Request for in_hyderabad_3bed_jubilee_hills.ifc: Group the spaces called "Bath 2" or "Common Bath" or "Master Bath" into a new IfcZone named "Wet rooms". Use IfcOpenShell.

First a look at what the model holds.

```python
import ifcopenshell

model = ifcopenshell.open("in_hyderabad_3bed_jubilee_hills.ifc")
print(model.schema)
seen = {}
for space in model.by_type("IfcSpace"):
    seen[space.LongName] = seen.get(space.LongName, 0) + 1
for name, count in sorted(seen.items(), key=str):
    print(count, "x", name)
print("zones:", [z.Name for z in model.by_type("IfcZone")][:20])
```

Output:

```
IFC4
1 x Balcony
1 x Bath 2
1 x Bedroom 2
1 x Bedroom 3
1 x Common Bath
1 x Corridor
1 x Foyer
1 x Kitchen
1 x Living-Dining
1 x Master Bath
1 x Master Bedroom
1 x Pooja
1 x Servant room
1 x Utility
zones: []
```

```python
import ifcopenshell
import ifcopenshell.api.group
import ifcopenshell.api.root

model = ifcopenshell.open("in_hyderabad_3bed_jubilee_hills.ifc")

names = {"Bath 2", "Common Bath", "Master Bath"}
spaces = [s for s in model.by_type("IfcSpace") if s.LongName in names]

zone = ifcopenshell.api.root.create_entity(model, ifc_class="IfcZone", name="Wet rooms")
ifcopenshell.api.group.assign_group(model, products=spaces, group=zone)
print(len(spaces), "spaces in", zone.Name)

model.write("in_hyderabad_3bed_jubilee_hills_edited.ifc")
```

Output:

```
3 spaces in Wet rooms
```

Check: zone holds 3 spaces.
